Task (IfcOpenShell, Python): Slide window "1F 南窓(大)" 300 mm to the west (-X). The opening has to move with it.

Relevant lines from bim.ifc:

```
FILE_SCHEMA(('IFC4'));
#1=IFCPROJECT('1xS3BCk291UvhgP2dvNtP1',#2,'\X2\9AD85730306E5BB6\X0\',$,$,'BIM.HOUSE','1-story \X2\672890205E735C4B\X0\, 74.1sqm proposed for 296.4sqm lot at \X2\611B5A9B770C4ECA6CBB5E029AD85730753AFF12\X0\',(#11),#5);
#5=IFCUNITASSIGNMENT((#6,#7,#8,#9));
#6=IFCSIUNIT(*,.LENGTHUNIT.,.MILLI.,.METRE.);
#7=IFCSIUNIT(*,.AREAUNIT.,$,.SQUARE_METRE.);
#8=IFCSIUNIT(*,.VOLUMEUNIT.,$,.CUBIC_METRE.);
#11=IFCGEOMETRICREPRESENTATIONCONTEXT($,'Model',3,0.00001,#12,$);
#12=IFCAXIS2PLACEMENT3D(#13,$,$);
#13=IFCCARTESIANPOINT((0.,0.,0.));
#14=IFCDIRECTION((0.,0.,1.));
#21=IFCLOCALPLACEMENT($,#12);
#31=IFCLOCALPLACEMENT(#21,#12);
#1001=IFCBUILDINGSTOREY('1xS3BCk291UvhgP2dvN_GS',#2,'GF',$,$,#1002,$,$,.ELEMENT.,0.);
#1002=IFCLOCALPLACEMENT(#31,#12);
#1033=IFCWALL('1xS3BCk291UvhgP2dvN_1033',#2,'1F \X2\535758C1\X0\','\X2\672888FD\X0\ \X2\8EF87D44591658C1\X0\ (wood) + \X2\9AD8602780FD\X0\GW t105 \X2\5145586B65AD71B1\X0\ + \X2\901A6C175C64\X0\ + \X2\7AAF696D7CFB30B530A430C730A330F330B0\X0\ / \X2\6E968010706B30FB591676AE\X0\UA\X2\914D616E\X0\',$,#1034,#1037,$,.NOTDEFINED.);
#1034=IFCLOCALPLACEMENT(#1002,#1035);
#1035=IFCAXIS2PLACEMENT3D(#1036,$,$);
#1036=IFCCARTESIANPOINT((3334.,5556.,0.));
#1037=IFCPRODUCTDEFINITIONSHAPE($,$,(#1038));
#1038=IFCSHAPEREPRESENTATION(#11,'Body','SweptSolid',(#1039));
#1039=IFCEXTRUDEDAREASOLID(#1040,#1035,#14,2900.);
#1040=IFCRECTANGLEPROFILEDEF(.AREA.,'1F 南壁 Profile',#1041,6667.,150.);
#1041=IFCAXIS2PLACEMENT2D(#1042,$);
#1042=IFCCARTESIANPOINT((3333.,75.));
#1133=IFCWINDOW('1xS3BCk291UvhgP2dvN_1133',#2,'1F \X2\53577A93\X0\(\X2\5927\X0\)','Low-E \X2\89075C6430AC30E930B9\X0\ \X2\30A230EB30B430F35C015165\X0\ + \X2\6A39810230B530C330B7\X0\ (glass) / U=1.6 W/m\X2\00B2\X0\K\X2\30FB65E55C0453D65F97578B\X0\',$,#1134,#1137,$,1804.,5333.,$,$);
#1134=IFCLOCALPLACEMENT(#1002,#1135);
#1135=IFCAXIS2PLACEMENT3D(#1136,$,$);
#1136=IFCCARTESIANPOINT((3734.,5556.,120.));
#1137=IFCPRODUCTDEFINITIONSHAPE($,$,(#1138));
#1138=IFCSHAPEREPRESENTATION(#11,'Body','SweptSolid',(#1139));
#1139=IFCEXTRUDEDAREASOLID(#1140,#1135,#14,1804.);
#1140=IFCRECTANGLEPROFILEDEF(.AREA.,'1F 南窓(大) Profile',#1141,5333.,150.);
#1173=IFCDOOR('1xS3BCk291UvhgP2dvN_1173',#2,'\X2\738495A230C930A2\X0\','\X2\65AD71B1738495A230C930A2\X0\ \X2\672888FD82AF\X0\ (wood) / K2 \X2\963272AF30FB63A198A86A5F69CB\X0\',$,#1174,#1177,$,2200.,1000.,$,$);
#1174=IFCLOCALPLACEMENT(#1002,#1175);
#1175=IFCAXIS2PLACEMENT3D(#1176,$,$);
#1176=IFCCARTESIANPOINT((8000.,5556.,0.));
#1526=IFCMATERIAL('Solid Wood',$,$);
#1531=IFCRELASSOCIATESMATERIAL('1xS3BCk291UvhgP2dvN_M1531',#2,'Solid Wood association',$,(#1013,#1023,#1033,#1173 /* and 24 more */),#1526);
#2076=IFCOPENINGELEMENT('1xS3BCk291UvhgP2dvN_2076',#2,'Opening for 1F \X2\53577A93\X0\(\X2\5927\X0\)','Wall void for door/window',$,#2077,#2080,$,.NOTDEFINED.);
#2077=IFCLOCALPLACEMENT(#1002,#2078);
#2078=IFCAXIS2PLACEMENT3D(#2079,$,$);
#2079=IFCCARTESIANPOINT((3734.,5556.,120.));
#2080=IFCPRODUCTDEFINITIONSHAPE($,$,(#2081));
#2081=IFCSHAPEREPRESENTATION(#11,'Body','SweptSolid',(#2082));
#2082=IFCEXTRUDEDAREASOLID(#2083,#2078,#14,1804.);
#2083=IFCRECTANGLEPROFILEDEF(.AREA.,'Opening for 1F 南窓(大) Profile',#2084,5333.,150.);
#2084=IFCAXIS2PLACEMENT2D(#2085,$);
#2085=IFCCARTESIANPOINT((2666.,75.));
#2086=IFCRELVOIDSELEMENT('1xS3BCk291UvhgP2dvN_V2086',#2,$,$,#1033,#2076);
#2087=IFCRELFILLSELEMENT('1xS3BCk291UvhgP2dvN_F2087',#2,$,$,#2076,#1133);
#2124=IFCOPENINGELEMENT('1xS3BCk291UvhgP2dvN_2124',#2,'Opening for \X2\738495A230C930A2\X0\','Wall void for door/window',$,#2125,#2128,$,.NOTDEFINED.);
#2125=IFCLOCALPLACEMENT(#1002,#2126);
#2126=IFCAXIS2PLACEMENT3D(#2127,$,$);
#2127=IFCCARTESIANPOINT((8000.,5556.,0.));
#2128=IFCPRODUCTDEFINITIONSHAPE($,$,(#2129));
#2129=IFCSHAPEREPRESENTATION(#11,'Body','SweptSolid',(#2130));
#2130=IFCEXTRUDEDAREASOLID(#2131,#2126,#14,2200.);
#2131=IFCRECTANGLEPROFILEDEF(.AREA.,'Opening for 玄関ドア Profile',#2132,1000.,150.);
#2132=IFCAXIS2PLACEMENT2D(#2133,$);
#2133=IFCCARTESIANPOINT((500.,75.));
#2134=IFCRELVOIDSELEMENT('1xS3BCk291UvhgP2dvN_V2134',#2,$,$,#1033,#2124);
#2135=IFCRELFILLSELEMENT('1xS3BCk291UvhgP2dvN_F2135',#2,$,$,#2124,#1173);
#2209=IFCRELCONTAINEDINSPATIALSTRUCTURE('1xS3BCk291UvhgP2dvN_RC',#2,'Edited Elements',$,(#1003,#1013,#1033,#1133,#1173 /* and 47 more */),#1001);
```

```python
import ifcopenshell
import ifcopenshell.api.geometry
import ifcopenshell.util.placement
import ifcopenshell.util.unit

model = ifcopenshell.open("bim.ifc")
unit_scale = ifcopenshell.util.unit.calculate_unit_scale(model)

window = model.by_id(1133)
opening = window.FillsVoids[0].RelatingOpeningElement
wall = opening.VoidsElements[0].RelatingBuildingElement

wall_matrix = ifcopenshell.util.placement.get_local_placement(wall.ObjectPlacement)
shift = wall_matrix[:3, 0] * -0.3 / unit_scale
before = ifcopenshell.util.placement.get_local_placement(window.ObjectPlacement)[:3, 3].copy()

# The window is not placed relative to its opening, so move both.
for product in (opening, window):
    matrix = ifcopenshell.util.placement.get_local_placement(product.ObjectPlacement)
    matrix[:3, 3] += shift
    ifcopenshell.api.geometry.edit_object_placement(model, product=product, matrix=matrix, is_si=False)

after = ifcopenshell.util.placement.get_local_placement(window.ObjectPlacement)[:3, 3]
print("window moved by", (after - before).round(3) + 0.0)

model.write("bim_edited.ifc")
```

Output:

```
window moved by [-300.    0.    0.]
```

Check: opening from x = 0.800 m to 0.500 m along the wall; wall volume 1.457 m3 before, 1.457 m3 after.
